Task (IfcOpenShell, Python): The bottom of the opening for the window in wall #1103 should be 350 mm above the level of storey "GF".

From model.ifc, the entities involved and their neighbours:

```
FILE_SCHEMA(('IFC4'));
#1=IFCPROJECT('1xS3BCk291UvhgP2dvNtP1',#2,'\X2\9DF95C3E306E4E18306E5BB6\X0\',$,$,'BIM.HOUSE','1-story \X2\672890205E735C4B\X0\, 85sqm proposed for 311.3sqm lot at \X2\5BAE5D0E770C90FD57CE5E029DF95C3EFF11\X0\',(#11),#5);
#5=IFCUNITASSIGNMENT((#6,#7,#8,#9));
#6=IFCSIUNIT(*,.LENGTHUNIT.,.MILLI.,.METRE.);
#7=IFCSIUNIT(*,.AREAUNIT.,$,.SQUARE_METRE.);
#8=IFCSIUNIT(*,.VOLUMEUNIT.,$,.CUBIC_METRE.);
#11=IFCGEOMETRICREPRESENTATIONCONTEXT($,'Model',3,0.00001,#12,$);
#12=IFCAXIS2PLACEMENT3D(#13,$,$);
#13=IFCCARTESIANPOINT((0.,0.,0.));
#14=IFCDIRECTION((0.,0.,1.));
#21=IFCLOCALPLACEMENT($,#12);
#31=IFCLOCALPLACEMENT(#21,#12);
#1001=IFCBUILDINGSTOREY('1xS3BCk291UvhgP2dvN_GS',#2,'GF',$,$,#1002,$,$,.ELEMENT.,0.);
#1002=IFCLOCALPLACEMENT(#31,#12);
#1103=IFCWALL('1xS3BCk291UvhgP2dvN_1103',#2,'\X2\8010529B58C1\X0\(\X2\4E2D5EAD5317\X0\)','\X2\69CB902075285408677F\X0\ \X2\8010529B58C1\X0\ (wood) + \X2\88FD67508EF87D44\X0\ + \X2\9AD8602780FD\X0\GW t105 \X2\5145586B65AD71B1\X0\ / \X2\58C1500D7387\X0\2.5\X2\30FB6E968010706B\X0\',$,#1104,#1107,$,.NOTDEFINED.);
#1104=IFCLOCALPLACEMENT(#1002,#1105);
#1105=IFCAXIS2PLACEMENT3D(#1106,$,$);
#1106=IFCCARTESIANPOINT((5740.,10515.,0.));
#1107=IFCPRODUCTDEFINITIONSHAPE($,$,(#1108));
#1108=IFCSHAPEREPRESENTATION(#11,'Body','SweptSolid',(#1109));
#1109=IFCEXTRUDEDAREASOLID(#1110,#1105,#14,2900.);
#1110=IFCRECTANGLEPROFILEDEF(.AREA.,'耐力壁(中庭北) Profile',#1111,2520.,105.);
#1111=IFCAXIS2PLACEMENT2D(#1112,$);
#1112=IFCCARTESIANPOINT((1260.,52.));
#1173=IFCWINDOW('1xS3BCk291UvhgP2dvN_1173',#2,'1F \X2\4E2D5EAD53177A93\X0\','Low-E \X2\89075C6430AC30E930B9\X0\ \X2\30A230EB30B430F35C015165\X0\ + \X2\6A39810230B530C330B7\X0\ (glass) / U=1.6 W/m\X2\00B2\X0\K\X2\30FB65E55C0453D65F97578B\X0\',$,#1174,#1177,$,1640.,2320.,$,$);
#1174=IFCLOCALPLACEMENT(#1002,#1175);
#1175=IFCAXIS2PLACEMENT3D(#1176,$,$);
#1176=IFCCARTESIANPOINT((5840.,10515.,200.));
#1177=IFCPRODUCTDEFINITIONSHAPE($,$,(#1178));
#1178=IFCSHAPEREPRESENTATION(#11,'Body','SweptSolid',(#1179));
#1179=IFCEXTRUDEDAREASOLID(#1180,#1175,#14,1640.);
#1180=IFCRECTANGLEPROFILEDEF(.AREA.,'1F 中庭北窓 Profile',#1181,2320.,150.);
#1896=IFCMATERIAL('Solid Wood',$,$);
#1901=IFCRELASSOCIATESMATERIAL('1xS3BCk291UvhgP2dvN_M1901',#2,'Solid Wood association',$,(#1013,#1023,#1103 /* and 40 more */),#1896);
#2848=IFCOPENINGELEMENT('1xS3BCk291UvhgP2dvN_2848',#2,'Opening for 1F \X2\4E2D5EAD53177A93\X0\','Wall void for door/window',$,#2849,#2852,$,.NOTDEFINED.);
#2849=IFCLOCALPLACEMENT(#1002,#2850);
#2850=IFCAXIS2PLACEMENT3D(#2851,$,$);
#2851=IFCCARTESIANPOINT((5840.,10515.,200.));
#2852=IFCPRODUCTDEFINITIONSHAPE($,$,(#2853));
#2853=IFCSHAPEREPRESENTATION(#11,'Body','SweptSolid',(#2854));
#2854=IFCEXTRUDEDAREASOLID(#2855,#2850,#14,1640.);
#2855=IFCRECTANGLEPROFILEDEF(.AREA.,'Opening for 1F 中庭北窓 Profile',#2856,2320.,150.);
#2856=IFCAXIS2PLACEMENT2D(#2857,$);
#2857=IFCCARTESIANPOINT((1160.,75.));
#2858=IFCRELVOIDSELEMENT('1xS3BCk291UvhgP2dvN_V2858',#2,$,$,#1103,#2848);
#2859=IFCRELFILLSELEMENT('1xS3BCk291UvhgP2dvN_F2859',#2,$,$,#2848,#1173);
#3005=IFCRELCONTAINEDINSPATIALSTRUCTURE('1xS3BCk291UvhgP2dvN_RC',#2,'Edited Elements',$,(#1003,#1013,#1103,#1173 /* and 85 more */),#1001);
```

```python
import numpy as np
import ifcopenshell
import ifcopenshell.api.geometry
import ifcopenshell.geom
import ifcopenshell.util.element
import ifcopenshell.util.placement
import ifcopenshell.util.shape
import ifcopenshell.util.unit

model = ifcopenshell.open("model.ifc")
unit_scale = ifcopenshell.util.unit.calculate_unit_scale(model)

window = model.by_id(1173)
opening = window.FillsVoids[0].RelatingOpeningElement
storey = ifcopenshell.util.element.get_container(window, ifc_class="IfcBuildingStorey")
level = ifcopenshell.util.placement.get_local_placement(storey.ObjectPlacement)[2, 3]

# The opening's origin need not be at the sill, so measure its lowest point.
shape = ifcopenshell.geom.create_shape(ifcopenshell.geom.settings(), opening)
bottom = ifcopenshell.util.shape.get_shape_bottom_elevation(shape, shape.geometry) / unit_scale
dz = level + 0.35 / unit_scale - bottom

shift = np.array([0.0, 0.0, dz])
# The window is not placed relative to its opening, so move both.
for product in (opening, window):
    matrix = ifcopenshell.util.placement.get_local_placement(product.ObjectPlacement)
    matrix[:3, 3] += shift
    ifcopenshell.api.geometry.edit_object_placement(model, product=product, matrix=matrix, is_si=False)

print(f"moved by {dz * unit_scale:+.3f} m")

model.write("model_edited.ifc")
```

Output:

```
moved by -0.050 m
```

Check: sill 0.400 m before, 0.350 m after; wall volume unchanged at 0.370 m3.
